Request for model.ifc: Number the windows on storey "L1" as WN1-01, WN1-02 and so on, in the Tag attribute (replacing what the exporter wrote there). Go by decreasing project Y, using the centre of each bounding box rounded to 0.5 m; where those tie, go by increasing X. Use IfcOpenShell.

First a look at what the model holds.

```python
import ifcopenshell
import ifcopenshell.util.element
import ifcopenshell.util.placement

model = ifcopenshell.open("model.ifc")
print(model.schema)
storey = next(s for s in model.by_type("IfcBuildingStorey") if s.Name == "L1")
windows = [e for e in ifcopenshell.util.element.get_decomposition(storey) if e.is_a("IfcWindow")]
for e in sorted(windows, key=lambda e: e.id()):
    origin = ifcopenshell.util.placement.get_local_placement(e.ObjectPlacement)[:3, 3]
    print(e.id(), e.Tag, e.Name, origin.round(2) + 0.0, sep=" | ")
```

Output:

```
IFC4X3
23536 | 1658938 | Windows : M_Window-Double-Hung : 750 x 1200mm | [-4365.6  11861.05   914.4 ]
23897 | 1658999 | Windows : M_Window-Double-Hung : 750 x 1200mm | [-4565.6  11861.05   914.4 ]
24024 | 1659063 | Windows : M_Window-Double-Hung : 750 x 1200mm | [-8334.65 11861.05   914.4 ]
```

```python
import ifcopenshell
import ifcopenshell.geom
import ifcopenshell.util.element
import ifcopenshell.util.shape

model = ifcopenshell.open("model.ifc")
settings = ifcopenshell.geom.settings()
settings.set("use-world-coords", True)


def centre(element):
    shape = ifcopenshell.geom.create_shape(settings, element)
    return ifcopenshell.util.shape.get_bbox_centroid(shape.geometry)


storey = next(s for s in model.by_type("IfcBuildingStorey") if s.Name == "L1")
windows = [e for e in ifcopenshell.util.element.get_decomposition(storey) if e.is_a("IfcWindow")]

# Insertion points can sit at a corner or the storey origin, so sort by the geometry (in metres).
centres = {e: centre(e) for e in windows}
windows.sort(key=lambda e: (-round(centres[e][1] / 0.5), centres[e][0]))

for i, e in enumerate(windows, start=1):
    number = f"WN1-{i:02d}"
    e.Tag = number
    print(e.id(), number)

model.write("model_updated.ifc")
```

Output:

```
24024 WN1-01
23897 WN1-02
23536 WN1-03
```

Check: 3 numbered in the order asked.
